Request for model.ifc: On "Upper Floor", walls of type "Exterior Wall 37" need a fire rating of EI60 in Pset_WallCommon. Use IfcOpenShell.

First a look at what the model holds.

```python
import ifcopenshell
import ifcopenshell.util.element

model = ifcopenshell.open("model.ifc")
print(model.schema)
storey = next(s for s in model.by_type("IfcBuildingStorey") if s.Name == "Upper Floor")
walls = [e for e in ifcopenshell.util.element.get_decomposition(storey) if e.is_a("IfcWall")]
seen = {}
for e in walls:
    element_type = ifcopenshell.util.element.get_type(e)
    key = (element_type.Name if element_type != e and element_type else None, ifcopenshell.util.element.get_pset(e, "Pset_WallCommon", "FireRating"))
    seen[key] = seen.get(key, 0) + 1
for (name, value), count in sorted(seen.items(), key=str):
    print(count, "x", name, "|", value)
```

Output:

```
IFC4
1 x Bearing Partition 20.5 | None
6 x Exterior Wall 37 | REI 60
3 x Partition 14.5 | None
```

```python
import ifcopenshell
import ifcopenshell.api.pset
import ifcopenshell.util.element

model = ifcopenshell.open("model.ifc")

storey = next(s for s in model.by_type("IfcBuildingStorey") if s.Name == "Upper Floor")
walls = [e for e in ifcopenshell.util.element.get_decomposition(storey) if e.is_a("IfcWall")]

count = 0
for e in walls:
    element_type = ifcopenshell.util.element.get_type(e)
    if element_type in (None, e) or element_type.Name != "Exterior Wall 37":
        continue
    # add_pset returns the element's existing set when there is one.
    pset = ifcopenshell.api.pset.add_pset(model, product=e, name="Pset_WallCommon")
    ifcopenshell.api.pset.edit_pset(model, pset=pset, properties={"FireRating": "EI60"})
    count += 1

print(count, "walls updated")

model.write("model_v2.ifc")
```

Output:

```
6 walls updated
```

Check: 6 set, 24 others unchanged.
